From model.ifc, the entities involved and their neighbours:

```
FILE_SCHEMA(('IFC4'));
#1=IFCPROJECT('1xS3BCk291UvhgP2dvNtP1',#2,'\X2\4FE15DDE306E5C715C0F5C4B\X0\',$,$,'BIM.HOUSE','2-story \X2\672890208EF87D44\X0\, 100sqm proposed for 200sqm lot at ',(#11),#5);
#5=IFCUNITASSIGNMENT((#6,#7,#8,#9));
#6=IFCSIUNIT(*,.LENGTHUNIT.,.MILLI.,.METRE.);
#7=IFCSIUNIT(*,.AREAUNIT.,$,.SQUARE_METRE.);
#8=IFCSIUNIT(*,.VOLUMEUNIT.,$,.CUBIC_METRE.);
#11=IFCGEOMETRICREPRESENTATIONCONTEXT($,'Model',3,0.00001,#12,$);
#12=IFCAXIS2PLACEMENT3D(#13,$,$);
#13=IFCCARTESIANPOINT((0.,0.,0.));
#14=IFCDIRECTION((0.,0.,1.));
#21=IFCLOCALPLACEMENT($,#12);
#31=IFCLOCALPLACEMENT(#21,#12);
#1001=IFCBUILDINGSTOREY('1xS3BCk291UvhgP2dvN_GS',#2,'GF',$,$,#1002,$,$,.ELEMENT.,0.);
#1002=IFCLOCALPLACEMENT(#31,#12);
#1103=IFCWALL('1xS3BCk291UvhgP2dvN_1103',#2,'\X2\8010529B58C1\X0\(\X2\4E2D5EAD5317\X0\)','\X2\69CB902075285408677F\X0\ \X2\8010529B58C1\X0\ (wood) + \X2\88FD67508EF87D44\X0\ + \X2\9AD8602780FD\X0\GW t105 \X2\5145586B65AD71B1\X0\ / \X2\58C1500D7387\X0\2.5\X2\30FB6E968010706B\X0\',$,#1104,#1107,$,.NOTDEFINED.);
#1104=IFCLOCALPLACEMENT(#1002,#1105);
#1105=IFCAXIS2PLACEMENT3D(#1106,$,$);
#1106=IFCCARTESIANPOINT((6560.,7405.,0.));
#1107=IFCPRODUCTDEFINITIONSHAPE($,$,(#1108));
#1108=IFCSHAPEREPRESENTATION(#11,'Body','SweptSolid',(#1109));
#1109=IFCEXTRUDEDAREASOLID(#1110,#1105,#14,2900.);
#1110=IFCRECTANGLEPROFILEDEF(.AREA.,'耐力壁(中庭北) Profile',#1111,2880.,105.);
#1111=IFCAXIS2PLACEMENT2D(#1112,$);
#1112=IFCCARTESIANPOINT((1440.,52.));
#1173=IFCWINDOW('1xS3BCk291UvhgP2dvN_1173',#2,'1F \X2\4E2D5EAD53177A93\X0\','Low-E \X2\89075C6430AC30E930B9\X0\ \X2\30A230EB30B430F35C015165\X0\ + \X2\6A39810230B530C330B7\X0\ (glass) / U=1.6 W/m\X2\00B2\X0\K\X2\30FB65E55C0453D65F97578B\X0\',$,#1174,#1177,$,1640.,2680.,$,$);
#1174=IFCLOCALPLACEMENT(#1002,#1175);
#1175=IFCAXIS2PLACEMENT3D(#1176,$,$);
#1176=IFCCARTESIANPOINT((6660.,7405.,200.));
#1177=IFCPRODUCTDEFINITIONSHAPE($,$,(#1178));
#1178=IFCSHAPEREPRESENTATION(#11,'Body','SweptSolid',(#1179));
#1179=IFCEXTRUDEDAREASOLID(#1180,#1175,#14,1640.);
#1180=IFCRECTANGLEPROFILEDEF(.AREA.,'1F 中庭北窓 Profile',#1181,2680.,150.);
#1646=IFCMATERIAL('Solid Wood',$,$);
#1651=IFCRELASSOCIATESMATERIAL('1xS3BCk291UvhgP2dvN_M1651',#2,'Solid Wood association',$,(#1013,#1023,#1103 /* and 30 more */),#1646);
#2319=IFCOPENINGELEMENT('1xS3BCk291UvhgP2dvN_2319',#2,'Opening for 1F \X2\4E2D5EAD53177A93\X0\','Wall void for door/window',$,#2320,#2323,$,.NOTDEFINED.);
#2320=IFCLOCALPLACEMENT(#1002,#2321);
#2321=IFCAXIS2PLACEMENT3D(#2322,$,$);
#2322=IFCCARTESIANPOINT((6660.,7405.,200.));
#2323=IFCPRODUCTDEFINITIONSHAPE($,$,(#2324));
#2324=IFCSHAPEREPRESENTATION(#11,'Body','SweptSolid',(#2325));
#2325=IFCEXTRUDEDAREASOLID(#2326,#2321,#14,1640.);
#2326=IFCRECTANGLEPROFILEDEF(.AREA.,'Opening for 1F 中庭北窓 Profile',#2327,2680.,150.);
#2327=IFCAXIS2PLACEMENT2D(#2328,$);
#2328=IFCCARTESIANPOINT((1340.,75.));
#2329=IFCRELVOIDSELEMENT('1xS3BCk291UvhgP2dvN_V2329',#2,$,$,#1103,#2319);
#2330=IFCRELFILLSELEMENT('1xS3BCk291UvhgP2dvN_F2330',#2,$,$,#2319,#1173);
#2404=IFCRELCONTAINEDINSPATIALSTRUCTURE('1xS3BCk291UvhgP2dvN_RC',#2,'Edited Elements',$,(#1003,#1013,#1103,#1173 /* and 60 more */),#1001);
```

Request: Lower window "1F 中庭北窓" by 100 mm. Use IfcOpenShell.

```python
import numpy as np
import ifcopenshell
import ifcopenshell.api.geometry
import ifcopenshell.util.placement
import ifcopenshell.util.unit

model = ifcopenshell.open("model.ifc")
unit_scale = ifcopenshell.util.unit.calculate_unit_scale(model)

window = model.by_guid("1xS3BCk291UvhgP2dvN_1173")
opening = window.FillsVoids[0].RelatingOpeningElement
dz = -0.1 / unit_scale

shift = np.array([0.0, 0.0, dz])
# The window is not placed relative to its opening, so move both.
for product in (opening, window):
    matrix = ifcopenshell.util.placement.get_local_placement(product.ObjectPlacement)
    matrix[:3, 3] += shift
    ifcopenshell.api.geometry.edit_object_placement(model, product=product, matrix=matrix, is_si=False)

print(f"moved by {dz * unit_scale:+.3f} m")

model.write("model_updated.ifc")
```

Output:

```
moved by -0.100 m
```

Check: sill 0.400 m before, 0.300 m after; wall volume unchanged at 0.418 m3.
